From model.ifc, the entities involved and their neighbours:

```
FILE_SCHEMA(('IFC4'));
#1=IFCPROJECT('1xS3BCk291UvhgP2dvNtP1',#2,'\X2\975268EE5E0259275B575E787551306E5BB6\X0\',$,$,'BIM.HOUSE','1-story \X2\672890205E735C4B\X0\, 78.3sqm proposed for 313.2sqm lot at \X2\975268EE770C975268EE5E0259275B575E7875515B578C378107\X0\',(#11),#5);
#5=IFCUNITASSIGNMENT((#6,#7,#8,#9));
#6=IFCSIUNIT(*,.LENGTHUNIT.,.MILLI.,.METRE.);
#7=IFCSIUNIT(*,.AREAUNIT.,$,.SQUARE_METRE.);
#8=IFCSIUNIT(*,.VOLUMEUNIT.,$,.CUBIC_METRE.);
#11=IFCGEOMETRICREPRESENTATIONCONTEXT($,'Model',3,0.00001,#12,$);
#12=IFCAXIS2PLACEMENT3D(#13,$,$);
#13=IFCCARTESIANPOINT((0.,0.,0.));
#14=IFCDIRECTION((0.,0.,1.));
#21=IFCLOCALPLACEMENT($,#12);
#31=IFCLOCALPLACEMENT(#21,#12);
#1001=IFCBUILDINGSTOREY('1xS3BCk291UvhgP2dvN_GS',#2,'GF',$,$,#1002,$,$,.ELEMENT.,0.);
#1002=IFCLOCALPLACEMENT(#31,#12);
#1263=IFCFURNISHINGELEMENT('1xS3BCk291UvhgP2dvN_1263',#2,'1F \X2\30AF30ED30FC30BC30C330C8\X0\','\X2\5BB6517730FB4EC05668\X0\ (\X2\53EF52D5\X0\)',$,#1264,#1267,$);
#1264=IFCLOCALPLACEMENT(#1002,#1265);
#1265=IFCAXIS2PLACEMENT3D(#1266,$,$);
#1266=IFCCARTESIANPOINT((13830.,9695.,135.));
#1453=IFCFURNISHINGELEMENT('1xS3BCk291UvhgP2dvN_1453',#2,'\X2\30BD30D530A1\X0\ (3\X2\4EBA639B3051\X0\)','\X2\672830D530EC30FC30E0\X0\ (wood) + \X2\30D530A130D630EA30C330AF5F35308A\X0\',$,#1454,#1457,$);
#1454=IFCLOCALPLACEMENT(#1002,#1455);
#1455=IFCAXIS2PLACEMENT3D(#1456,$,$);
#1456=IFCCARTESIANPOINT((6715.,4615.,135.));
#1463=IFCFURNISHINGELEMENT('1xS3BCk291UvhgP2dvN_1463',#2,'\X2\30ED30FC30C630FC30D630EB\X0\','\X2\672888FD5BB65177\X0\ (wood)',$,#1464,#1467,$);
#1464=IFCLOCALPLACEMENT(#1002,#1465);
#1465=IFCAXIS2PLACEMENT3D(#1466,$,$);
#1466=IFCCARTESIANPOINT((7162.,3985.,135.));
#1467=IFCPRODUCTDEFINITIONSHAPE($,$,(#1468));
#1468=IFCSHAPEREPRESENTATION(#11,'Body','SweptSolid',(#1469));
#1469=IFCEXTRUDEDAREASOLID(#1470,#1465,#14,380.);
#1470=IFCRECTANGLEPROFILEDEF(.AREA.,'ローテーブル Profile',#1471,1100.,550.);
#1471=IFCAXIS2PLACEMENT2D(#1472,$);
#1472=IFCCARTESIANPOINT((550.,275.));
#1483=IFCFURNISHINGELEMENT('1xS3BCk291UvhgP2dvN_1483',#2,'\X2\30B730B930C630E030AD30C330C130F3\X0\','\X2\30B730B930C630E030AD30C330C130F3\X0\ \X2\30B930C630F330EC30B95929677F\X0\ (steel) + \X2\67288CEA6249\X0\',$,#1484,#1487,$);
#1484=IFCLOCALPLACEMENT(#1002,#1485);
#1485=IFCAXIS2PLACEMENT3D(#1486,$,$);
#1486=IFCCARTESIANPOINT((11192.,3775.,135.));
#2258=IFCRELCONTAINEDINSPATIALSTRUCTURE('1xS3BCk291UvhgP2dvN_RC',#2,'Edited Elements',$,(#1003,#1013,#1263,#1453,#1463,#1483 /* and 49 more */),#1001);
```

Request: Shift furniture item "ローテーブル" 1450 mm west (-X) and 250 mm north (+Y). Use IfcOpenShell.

```python
import ifcopenshell
import ifcopenshell.api.geometry
import ifcopenshell.util.placement
import ifcopenshell.util.unit

model = ifcopenshell.open("model.ifc")
unit_scale = ifcopenshell.util.unit.calculate_unit_scale(model)

item = model.by_guid("1xS3BCk291UvhgP2dvN_1463")
matrix = ifcopenshell.util.placement.get_local_placement(item.ObjectPlacement)
matrix[0, 3] -= 1.45 / unit_scale
matrix[1, 3] += 0.25 / unit_scale
ifcopenshell.api.geometry.edit_object_placement(model, product=item, matrix=matrix, is_si=False)

print(ifcopenshell.util.placement.get_local_placement(item.ObjectPlacement).round(3) + 0.0)

model.write("model_v2.ifc")
```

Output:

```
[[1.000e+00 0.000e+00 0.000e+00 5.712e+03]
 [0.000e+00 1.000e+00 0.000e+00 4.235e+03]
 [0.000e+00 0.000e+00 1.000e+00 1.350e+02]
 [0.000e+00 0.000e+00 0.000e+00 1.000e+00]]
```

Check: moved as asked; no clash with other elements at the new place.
